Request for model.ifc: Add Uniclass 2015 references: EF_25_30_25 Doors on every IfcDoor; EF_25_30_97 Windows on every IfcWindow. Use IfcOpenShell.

First a look at what the model holds.

```python
import ifcopenshell

model = ifcopenshell.open("model.ifc")
print(model.schema)
print("classifications:", [c.Name for c in model.by_type("IfcClassification")])
for ifc_class in ("IfcDoor", "IfcRoof", "IfcStair", "IfcWall", "IfcWindow"):
    print(ifc_class, len(model.by_type(ifc_class)))
```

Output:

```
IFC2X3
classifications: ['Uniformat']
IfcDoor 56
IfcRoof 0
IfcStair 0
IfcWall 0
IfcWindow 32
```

```python
import ifcopenshell
import ifcopenshell.api.classification

model = ifcopenshell.open("model.ifc")

# IFC2X3 requires Source and Edition and has no link from the project to the system.
system = model.create_entity("IfcClassification", Source="NBS", Edition="2015", Name="Uniclass 2015")

codes = {
    "IfcDoor": ("EF_25_30_25", "Doors"),
    "IfcWindow": ("EF_25_30_97", "Windows"),
}
for ifc_class, (code, name) in codes.items():
    products = model.by_type(ifc_class)
    ifcopenshell.api.classification.add_reference(
        model, products=products, classification=system, identification=code, name=name
    )
    print(code, len(products))

model.write("model_updated.ifc")
```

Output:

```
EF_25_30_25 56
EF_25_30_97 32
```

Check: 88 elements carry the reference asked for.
